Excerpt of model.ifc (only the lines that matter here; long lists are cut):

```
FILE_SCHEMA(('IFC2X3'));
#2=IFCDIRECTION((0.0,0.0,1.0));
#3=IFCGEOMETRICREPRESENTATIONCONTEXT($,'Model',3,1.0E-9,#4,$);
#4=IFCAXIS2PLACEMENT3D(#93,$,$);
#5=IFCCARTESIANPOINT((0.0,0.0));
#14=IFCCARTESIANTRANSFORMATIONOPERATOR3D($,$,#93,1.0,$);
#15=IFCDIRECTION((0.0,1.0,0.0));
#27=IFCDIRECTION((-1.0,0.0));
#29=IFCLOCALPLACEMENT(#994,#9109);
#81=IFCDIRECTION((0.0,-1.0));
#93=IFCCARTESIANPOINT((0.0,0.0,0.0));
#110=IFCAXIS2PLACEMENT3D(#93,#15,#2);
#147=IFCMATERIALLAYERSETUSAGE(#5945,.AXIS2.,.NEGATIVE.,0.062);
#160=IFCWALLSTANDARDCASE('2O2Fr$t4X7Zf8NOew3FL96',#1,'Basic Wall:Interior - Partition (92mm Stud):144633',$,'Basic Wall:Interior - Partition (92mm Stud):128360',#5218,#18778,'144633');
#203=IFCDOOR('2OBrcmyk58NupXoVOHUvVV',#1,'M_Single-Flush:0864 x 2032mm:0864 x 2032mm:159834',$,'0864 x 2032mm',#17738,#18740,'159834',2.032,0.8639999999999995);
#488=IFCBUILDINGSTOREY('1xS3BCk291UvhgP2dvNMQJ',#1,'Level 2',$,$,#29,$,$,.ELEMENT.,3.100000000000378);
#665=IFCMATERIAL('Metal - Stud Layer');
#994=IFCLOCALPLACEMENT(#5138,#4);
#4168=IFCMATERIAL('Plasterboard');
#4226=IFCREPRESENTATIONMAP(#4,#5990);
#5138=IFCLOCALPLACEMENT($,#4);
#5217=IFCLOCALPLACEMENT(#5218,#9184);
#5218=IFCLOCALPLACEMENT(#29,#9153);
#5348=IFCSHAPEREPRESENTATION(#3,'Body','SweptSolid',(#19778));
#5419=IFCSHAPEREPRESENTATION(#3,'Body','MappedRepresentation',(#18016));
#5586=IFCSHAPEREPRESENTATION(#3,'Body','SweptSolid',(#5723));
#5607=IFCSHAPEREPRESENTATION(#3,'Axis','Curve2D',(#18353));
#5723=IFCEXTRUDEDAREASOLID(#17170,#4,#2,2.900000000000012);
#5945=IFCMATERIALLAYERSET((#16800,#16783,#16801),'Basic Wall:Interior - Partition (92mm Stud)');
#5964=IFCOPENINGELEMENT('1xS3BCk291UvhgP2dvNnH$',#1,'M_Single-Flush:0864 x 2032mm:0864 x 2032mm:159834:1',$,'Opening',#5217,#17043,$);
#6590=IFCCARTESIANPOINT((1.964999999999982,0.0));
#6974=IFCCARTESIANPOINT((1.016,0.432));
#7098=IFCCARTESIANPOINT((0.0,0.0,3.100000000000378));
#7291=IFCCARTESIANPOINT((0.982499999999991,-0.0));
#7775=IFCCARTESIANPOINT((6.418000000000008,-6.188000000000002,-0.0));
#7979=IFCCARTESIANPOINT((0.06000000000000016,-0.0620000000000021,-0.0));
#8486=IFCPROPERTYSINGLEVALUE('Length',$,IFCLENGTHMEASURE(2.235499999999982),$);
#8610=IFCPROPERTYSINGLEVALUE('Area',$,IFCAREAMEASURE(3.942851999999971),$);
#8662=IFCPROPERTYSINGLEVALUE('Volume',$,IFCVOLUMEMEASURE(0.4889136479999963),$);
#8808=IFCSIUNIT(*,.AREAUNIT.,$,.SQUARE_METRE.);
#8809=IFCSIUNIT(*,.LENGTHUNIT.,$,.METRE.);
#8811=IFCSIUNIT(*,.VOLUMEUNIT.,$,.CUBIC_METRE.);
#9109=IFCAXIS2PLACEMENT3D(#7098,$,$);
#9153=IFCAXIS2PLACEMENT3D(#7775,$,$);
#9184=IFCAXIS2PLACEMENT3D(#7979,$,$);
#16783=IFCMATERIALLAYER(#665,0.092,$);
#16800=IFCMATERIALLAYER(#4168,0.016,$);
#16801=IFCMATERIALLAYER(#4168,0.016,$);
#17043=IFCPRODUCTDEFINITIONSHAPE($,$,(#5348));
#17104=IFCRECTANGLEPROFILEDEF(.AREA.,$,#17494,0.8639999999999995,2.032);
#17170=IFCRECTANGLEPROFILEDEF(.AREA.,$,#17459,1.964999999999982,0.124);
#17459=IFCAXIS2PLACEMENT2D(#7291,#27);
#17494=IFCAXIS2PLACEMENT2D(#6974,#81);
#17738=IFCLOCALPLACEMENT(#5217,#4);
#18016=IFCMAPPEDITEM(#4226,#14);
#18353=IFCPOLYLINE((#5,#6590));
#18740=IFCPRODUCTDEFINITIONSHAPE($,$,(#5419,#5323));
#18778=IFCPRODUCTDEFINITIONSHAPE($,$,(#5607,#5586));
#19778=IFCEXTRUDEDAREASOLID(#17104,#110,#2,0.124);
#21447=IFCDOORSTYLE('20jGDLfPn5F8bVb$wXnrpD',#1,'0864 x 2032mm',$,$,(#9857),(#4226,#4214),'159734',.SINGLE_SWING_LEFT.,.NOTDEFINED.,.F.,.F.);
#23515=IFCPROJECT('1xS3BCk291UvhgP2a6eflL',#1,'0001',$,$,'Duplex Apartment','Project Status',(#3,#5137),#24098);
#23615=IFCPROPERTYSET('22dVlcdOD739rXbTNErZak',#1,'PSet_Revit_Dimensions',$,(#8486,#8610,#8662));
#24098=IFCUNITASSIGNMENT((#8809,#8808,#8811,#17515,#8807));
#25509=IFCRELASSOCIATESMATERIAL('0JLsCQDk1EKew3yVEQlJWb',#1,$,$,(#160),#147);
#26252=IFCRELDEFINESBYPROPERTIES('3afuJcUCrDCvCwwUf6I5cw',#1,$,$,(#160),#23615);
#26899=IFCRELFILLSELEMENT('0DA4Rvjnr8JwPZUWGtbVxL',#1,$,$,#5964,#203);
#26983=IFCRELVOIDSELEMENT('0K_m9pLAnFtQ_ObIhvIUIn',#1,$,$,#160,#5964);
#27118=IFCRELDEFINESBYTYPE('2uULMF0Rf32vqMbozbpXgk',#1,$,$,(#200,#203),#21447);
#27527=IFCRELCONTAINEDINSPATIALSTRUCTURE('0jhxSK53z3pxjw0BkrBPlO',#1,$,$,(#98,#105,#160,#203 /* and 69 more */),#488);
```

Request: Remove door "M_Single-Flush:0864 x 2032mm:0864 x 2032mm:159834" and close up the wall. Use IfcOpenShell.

```python
import ifcopenshell
import ifcopenshell.api.feature
import ifcopenshell.api.pset
import ifcopenshell.api.root
import ifcopenshell.geom
import ifcopenshell.util.element
import ifcopenshell.util.shape
import ifcopenshell.util.unit

model = ifcopenshell.open("model.ifc")
area_scale = ifcopenshell.util.unit.calculate_unit_scale(model, "AREAUNIT")
volume_scale = ifcopenshell.util.unit.calculate_unit_scale(model, "VOLUMEUNIT")
settings = ifcopenshell.geom.settings()


def volume(element):
    """Net volume in cubic metres, openings subtracted."""
    shape = ifcopenshell.geom.create_shape(settings, element)
    return ifcopenshell.util.shape.get_volume(shape.geometry)


door = model.by_id(203)
opening = door.FillsVoids[0].RelatingOpeningElement
wall = opening.VoidsElements[0].RelatingBuildingElement
before = volume(wall)

ifcopenshell.api.root.remove_product(model, product=door)
ifcopenshell.api.feature.remove_feature(model, feature=opening)

after = volume(wall)
thickness = 0.124  # wall thickness in metres

# Update the wall's stored quantities.
pset = model.by_id(ifcopenshell.util.element.get_pset(wall, "PSet_Revit_Dimensions", should_inherit=False)["id"])
ifcopenshell.api.pset.edit_pset(model, pset=pset, properties={
    "Area": model.create_entity("IfcAreaMeasure", after / thickness / area_scale),
    "Volume": model.create_entity("IfcVolumeMeasure", after / volume_scale),
})

print(f"wall volume {before:.3f} -> {after:.3f} m3")

model.write("model_v2.ifc")
```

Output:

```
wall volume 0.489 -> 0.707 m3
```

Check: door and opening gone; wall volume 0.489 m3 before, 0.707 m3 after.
